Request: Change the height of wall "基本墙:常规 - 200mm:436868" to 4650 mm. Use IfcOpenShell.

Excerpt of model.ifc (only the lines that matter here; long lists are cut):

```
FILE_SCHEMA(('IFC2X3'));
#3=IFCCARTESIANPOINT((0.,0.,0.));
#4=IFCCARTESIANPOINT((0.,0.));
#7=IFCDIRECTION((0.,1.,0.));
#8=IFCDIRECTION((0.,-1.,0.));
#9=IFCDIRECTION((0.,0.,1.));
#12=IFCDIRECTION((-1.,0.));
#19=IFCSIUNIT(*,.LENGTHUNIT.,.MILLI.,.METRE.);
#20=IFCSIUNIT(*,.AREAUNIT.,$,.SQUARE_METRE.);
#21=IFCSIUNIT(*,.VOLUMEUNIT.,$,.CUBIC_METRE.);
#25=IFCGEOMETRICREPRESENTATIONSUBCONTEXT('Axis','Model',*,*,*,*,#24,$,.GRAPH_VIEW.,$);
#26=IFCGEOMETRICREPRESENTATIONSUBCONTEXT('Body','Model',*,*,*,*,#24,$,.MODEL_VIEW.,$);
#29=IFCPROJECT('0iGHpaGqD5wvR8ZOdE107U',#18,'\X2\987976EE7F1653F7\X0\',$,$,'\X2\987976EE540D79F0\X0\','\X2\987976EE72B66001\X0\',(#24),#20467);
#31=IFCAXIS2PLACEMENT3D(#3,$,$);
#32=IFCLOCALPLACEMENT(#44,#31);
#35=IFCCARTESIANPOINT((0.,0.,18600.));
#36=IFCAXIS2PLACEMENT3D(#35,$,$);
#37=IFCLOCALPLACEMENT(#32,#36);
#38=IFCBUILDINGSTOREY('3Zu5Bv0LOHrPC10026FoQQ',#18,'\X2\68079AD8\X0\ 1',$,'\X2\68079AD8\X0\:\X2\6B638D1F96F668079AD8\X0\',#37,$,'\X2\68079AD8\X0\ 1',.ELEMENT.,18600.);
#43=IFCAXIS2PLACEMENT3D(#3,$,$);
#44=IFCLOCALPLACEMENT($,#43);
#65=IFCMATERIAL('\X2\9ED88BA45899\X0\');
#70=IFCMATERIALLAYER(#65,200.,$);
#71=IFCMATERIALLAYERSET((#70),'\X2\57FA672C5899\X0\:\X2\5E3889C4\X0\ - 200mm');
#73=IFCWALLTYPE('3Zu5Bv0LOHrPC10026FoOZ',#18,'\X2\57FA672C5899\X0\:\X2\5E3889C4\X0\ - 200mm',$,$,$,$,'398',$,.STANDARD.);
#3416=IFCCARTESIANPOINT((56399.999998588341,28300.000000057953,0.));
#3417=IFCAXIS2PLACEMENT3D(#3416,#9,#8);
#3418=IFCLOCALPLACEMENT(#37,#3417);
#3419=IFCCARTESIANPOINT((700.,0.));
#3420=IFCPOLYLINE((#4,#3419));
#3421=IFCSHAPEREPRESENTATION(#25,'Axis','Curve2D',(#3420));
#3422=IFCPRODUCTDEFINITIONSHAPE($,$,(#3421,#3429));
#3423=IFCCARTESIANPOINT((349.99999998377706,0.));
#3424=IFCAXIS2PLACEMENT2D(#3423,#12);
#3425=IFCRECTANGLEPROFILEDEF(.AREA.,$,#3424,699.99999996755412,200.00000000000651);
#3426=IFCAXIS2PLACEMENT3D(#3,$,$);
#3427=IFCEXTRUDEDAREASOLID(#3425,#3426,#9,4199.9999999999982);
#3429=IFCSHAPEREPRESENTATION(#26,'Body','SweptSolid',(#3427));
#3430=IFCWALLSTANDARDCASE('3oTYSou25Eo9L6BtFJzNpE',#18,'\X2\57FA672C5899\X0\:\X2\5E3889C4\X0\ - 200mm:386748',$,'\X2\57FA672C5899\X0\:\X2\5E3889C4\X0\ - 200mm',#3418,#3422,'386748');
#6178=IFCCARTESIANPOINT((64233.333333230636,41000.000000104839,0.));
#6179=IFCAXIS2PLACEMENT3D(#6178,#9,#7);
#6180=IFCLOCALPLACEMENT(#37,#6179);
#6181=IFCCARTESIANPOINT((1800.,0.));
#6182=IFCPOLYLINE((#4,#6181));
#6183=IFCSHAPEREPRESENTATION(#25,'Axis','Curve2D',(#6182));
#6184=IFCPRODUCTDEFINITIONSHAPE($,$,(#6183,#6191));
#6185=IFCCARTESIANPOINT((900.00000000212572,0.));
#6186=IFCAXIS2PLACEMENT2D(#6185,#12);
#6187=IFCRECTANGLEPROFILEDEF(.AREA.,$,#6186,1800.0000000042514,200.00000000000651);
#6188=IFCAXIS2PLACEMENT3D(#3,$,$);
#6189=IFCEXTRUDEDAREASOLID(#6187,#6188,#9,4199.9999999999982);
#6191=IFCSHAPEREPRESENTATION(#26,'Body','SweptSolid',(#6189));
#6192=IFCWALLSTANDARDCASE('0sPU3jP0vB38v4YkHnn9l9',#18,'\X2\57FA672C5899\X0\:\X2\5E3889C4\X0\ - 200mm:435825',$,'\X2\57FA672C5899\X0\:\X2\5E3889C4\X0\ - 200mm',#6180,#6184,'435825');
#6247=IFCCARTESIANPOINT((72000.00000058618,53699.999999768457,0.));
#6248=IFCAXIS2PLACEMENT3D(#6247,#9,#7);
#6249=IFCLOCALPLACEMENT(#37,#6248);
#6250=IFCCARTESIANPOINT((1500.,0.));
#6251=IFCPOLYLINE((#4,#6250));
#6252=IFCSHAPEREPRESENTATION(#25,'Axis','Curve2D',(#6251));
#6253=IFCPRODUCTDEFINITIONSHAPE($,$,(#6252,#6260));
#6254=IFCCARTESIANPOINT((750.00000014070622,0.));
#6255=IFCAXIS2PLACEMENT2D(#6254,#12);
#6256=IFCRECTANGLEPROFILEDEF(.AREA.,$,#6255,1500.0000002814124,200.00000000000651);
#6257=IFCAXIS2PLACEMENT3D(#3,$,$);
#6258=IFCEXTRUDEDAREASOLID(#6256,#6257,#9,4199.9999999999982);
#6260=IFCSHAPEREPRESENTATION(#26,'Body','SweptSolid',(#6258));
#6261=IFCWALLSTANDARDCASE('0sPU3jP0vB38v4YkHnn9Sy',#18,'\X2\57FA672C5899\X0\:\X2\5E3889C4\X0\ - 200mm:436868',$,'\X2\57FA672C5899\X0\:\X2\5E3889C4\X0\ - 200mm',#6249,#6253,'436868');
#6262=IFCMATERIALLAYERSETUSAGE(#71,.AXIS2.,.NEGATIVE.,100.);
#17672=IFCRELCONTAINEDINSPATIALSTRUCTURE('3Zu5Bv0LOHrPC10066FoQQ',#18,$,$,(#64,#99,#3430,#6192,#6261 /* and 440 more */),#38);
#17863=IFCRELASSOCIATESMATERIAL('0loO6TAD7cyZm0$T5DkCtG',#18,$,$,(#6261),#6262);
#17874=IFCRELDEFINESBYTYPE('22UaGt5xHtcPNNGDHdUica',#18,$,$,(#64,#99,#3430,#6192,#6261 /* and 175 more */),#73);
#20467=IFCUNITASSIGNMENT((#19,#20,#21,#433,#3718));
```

```python
import ifcopenshell
import ifcopenshell.geom
import ifcopenshell.util.representation
import ifcopenshell.util.shape

model = ifcopenshell.open("model.ifc")
settings = ifcopenshell.geom.settings()


def volume(element):
    """Net volume in cubic metres, openings subtracted."""
    shape = ifcopenshell.geom.create_shape(settings, element)
    return ifcopenshell.util.shape.get_volume(shape.geometry)


wall = model.by_id(6261)
before = volume(wall)

body = ifcopenshell.util.representation.get_representation(wall, "Model", "Body")
solid = body.Items[0]
old_height = solid.Depth
solid.Depth = 4650.0
after = volume(wall)

print(f"height {old_height:g} -> {solid.Depth:g}, volume {before:.3f} -> {after:.3f} m3")

model.write("model_v2.ifc")
```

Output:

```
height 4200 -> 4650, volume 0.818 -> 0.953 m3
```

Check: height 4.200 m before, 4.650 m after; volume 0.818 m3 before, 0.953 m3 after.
